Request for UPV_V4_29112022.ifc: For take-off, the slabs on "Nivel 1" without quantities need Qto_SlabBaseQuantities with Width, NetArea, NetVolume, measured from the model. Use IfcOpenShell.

First a look at what the model holds.

```python
import ifcopenshell
import ifcopenshell.util.element
import ifcopenshell.util.unit

model = ifcopenshell.open("UPV_V4_29112022.ifc")
print(model.schema)
for unit_type in ("LENGTHUNIT", "AREAUNIT", "VOLUMEUNIT"):
    print(unit_type, ifcopenshell.util.unit.calculate_unit_scale(model, unit_type))
storey = next(s for s in model.by_type("IfcBuildingStorey") if s.Name == "Nivel 1")
slabs = [e for e in ifcopenshell.util.element.get_decomposition(storey) if e.is_a("IfcSlab")]
for e in sorted(slabs, key=lambda e: e.id()):
    print(e.id(), e.is_a(), e.Name, list(ifcopenshell.util.element.get_psets(e, qtos_only=True)), sep=" | ")
```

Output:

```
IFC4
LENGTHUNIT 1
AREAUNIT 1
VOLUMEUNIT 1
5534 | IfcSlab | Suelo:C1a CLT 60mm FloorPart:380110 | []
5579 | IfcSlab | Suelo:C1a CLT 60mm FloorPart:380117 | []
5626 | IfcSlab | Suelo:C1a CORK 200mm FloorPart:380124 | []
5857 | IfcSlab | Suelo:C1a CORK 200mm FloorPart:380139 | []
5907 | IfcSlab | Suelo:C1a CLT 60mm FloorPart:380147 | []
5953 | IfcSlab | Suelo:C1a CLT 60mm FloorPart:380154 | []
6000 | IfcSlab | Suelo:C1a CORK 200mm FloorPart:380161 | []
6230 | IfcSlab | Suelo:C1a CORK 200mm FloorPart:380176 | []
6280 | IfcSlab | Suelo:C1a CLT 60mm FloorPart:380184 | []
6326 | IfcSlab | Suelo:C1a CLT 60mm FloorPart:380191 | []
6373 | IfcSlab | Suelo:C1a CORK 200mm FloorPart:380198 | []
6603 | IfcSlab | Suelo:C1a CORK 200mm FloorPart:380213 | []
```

```python
import ifcopenshell
import ifcopenshell.api.pset
import ifcopenshell.geom
import ifcopenshell.util.element
import ifcopenshell.util.shape
import ifcopenshell.util.unit

model = ifcopenshell.open("UPV_V4_29112022.ifc")
unit_scale = ifcopenshell.util.unit.calculate_unit_scale(model)
area_scale = ifcopenshell.util.unit.calculate_unit_scale(model, "AREAUNIT")
volume_scale = ifcopenshell.util.unit.calculate_unit_scale(model, "VOLUMEUNIT")
settings = ifcopenshell.geom.settings()

storey = next(s for s in model.by_type("IfcBuildingStorey") if s.Name == "Nivel 1")
slabs = [e for e in ifcopenshell.util.element.get_decomposition(storey) if e.is_a("IfcSlab")]

for e in sorted(slabs, key=lambda e: e.id()):
    if ifcopenshell.util.element.get_psets(e, qtos_only=True, should_inherit=False):
        continue
    # Geometry comes back in metres, in the element's own axes.
    shape = ifcopenshell.geom.create_shape(settings, e)
    values = {
        "Width": ifcopenshell.util.shape.get_z(shape.geometry) / unit_scale,
        "NetArea": ifcopenshell.util.shape.get_footprint_area(shape.geometry) / area_scale,
        "NetVolume": ifcopenshell.util.shape.get_volume(shape.geometry) / volume_scale,
    }
    qto = ifcopenshell.api.pset.add_qto(model, product=e, name="Qto_SlabBaseQuantities")
    ifcopenshell.api.pset.edit_qto(model, qto=qto, properties=values)
    print(e.id(), {k: round(v, 3) for k, v in values.items()})

model.write("UPV_V4_29112022_v2.ifc")
```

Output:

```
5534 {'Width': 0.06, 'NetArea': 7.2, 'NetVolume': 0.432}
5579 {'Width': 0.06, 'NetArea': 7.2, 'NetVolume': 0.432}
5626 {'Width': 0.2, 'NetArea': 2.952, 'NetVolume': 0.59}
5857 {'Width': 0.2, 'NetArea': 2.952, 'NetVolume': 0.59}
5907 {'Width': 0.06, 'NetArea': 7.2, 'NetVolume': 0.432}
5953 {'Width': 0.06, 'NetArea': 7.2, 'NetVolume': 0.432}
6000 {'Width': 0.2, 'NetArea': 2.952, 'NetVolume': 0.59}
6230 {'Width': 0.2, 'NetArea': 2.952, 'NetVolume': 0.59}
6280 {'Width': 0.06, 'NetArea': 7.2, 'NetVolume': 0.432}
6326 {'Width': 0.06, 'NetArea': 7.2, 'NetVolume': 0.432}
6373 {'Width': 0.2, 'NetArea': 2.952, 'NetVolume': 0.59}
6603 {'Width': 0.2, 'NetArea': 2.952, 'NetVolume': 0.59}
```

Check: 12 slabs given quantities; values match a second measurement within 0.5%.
